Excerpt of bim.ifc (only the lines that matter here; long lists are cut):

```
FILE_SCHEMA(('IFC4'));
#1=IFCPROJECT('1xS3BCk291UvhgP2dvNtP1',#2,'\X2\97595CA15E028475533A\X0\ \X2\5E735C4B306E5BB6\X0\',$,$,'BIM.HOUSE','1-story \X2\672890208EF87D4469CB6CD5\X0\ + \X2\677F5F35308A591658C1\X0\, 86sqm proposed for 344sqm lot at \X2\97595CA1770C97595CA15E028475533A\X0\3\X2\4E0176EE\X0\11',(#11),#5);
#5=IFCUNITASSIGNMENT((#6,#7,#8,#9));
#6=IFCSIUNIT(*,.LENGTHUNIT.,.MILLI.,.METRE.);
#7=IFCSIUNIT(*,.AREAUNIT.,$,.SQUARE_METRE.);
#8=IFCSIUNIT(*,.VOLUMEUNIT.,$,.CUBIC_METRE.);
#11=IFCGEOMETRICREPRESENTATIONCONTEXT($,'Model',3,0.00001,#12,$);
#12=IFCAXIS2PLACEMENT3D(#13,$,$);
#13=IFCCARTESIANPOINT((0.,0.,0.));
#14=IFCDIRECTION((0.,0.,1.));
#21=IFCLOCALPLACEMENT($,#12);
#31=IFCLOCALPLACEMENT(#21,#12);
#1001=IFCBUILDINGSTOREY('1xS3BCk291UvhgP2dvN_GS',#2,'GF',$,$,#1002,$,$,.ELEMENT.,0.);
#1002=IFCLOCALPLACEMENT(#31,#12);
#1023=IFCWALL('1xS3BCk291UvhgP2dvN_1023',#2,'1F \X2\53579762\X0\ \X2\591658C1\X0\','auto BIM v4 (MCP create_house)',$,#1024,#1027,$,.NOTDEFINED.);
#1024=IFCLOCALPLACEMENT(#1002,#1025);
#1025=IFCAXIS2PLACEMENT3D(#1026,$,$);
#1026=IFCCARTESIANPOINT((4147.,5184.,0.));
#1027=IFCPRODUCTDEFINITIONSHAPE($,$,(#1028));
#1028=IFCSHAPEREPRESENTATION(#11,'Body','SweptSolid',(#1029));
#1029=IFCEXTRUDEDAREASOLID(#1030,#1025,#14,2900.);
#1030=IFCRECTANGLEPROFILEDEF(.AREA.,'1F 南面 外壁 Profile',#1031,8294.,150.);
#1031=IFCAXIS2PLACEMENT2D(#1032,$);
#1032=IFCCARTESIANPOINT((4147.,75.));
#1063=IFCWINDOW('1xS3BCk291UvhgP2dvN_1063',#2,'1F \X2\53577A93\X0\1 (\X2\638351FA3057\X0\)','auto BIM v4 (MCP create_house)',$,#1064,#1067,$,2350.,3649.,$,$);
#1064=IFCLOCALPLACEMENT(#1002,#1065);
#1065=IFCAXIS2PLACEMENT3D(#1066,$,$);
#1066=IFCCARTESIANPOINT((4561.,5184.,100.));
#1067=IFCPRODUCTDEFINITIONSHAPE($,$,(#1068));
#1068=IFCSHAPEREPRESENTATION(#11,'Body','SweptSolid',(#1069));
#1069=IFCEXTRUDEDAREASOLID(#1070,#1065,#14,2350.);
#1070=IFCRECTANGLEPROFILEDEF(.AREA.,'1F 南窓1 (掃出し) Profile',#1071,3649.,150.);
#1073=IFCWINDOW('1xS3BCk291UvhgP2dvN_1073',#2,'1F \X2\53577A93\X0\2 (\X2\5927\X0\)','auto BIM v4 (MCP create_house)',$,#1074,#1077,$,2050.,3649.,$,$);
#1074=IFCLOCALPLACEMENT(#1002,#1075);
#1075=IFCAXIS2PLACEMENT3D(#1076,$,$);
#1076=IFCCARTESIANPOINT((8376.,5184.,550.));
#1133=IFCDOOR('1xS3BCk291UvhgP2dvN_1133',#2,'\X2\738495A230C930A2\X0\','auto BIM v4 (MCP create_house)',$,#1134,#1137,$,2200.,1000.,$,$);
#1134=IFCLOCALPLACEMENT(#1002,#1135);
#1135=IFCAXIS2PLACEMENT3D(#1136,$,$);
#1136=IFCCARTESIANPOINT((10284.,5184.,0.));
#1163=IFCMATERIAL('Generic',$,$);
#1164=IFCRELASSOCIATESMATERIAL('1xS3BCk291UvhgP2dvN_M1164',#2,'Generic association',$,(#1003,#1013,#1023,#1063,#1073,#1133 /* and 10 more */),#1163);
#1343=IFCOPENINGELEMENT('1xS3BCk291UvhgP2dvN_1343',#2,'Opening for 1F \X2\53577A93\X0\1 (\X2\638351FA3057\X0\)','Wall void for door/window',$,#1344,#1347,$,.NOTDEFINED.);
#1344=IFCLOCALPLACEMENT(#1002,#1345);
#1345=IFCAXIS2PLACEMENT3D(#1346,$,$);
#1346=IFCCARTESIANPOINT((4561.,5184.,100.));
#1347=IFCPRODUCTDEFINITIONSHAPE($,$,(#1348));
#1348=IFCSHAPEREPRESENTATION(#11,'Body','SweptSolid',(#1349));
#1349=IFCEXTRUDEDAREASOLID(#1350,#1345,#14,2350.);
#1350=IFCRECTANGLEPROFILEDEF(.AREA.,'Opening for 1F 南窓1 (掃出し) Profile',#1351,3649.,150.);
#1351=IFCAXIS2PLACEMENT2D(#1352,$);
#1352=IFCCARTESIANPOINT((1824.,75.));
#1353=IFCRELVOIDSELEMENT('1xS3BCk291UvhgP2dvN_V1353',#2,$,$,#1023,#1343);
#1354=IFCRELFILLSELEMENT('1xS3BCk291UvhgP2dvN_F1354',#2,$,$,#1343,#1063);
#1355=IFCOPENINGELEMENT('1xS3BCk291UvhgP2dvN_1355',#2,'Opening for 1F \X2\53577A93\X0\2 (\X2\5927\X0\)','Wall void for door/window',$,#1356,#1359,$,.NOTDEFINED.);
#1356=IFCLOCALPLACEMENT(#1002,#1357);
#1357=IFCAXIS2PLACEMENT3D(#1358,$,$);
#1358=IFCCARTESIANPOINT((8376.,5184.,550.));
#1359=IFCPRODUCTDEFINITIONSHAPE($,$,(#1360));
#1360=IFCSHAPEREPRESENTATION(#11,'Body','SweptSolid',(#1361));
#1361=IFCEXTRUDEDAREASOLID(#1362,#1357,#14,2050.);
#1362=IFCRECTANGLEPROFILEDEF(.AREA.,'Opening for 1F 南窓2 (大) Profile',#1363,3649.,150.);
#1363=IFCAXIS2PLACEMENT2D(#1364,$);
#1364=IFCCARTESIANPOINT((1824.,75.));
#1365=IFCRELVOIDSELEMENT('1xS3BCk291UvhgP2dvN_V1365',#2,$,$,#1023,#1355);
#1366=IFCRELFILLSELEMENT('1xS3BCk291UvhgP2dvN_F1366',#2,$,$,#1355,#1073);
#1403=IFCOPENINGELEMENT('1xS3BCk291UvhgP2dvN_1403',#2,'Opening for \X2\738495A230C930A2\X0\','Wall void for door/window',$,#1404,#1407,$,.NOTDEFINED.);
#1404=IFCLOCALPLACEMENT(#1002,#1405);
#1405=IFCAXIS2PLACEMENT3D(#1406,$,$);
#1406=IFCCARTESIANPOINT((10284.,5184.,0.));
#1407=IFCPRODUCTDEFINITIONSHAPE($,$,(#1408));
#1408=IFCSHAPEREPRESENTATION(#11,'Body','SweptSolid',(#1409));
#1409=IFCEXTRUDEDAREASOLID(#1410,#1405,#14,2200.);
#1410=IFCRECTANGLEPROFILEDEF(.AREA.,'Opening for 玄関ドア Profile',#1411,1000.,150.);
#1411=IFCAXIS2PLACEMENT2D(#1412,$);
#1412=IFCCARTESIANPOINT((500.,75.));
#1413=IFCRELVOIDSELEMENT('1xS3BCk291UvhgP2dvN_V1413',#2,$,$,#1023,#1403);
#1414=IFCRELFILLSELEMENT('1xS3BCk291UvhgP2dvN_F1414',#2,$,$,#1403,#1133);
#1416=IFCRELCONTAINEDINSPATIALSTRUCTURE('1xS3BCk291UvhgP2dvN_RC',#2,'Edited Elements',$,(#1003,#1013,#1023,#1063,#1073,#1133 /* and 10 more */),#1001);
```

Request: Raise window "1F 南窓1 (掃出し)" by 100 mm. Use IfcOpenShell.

```python
import numpy as np
import ifcopenshell
import ifcopenshell.api.geometry
import ifcopenshell.util.placement
import ifcopenshell.util.unit

model = ifcopenshell.open("bim.ifc")
unit_scale = ifcopenshell.util.unit.calculate_unit_scale(model)

window = model.by_id(1063)
opening = window.FillsVoids[0].RelatingOpeningElement
dz = 0.1 / unit_scale

shift = np.array([0.0, 0.0, dz])
# The window is not placed relative to its opening, so move both.
for product in (opening, window):
    matrix = ifcopenshell.util.placement.get_local_placement(product.ObjectPlacement)
    matrix[:3, 3] += shift
    ifcopenshell.api.geometry.edit_object_placement(model, product=product, matrix=matrix, is_si=False)

print(f"moved by {dz * unit_scale:+.3f} m")

model.write("bim-out.ifc")
```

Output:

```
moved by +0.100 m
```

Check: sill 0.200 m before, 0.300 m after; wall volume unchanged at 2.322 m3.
